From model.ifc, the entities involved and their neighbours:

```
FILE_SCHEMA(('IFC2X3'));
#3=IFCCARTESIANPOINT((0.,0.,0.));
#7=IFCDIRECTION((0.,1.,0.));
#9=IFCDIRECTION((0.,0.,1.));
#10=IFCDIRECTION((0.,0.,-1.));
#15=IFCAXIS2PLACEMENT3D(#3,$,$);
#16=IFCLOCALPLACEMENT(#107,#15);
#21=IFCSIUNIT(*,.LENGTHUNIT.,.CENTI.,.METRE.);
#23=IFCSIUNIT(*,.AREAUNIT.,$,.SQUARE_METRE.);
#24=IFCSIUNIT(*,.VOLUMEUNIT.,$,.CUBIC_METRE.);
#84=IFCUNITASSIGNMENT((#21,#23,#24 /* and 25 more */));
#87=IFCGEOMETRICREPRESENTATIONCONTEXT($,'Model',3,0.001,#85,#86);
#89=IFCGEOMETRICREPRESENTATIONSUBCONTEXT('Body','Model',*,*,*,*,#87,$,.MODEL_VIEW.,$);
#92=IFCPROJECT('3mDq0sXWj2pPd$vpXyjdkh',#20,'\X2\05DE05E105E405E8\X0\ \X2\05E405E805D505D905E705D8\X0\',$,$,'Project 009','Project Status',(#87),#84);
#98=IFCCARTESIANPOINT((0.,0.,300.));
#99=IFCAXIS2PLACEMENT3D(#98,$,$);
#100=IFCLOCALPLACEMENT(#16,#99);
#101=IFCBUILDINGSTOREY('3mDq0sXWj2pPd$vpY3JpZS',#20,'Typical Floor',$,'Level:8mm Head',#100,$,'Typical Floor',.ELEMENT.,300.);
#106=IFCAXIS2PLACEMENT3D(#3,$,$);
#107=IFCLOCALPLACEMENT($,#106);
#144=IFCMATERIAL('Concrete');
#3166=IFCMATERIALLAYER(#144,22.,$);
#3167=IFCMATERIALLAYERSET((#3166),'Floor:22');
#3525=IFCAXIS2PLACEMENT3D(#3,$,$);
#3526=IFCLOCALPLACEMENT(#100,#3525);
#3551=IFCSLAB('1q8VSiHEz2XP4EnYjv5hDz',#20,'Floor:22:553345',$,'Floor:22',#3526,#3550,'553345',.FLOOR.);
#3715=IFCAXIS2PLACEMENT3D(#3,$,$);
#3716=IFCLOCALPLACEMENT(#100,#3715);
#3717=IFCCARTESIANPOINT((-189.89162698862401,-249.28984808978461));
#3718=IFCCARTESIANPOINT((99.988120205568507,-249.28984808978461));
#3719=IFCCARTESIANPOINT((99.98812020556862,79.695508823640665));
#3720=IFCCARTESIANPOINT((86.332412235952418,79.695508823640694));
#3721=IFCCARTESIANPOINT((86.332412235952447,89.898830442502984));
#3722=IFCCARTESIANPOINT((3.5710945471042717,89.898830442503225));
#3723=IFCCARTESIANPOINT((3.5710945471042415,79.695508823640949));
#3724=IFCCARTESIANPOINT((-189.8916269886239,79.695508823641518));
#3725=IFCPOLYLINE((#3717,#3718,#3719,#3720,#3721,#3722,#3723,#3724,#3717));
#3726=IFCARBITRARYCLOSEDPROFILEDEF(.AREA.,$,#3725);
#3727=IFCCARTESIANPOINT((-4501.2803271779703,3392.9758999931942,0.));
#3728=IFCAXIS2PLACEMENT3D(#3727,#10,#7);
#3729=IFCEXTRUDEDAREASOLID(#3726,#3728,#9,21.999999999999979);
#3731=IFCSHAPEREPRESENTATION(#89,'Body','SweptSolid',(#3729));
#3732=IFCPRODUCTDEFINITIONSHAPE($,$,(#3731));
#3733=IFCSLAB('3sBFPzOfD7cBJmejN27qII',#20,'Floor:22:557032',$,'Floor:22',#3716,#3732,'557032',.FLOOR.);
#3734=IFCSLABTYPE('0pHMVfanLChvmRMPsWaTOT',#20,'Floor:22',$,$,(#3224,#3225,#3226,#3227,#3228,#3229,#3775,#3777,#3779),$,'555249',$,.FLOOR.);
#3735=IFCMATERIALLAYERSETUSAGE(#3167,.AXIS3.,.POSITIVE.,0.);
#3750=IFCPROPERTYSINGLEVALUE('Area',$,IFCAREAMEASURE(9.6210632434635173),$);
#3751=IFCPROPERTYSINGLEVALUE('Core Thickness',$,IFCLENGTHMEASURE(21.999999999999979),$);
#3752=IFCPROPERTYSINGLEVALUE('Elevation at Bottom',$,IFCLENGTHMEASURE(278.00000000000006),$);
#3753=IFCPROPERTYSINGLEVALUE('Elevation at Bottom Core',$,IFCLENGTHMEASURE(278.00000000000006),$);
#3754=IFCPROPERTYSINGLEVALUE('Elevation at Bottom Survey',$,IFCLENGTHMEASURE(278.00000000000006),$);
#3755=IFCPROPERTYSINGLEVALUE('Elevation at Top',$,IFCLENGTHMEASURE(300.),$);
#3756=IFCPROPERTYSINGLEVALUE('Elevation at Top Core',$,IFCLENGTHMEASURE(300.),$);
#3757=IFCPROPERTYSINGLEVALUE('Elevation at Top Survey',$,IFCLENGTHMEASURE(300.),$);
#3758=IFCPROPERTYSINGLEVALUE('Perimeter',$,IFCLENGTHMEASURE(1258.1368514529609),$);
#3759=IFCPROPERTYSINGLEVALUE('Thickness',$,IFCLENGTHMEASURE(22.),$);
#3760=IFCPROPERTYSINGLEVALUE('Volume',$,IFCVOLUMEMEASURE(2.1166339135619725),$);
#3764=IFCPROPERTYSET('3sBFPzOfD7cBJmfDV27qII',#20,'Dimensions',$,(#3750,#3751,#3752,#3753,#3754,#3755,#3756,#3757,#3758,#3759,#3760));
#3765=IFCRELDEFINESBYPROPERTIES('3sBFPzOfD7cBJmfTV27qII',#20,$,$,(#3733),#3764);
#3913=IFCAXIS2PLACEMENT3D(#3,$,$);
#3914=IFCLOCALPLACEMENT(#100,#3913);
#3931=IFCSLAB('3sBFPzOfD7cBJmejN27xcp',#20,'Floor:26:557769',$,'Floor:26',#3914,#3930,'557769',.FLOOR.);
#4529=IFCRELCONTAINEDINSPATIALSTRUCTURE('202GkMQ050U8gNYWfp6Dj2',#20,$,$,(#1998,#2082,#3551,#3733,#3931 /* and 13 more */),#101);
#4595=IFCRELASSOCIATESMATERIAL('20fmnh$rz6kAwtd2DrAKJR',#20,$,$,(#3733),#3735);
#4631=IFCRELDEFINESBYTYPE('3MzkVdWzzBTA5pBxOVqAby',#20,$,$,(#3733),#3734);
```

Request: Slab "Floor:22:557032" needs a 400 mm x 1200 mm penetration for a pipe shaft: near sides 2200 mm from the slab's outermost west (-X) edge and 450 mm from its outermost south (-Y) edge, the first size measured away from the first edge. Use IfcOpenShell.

```python
import numpy as np
import ifcopenshell
import ifcopenshell.api.feature
import ifcopenshell.api.geometry
import ifcopenshell.api.pset
import ifcopenshell.api.root
import ifcopenshell.geom
import ifcopenshell.util.element
import ifcopenshell.util.placement
import ifcopenshell.util.representation
import ifcopenshell.util.shape
import ifcopenshell.util.unit

model = ifcopenshell.open("model.ifc")
unit_scale = ifcopenshell.util.unit.calculate_unit_scale(model)
area_scale = ifcopenshell.util.unit.calculate_unit_scale(model, "AREAUNIT")
volume_scale = ifcopenshell.util.unit.calculate_unit_scale(model, "VOLUMEUNIT")
settings = ifcopenshell.geom.settings()


def volume(element):
    """Net volume in cubic metres, openings subtracted."""
    shape = ifcopenshell.geom.create_shape(settings, element)
    return ifcopenshell.util.shape.get_volume(shape.geometry)


slab = model.by_id(3733)
before = volume(slab)

# Extent in the slab's own axes, in metres. The edges named are its -X and -Y sides.
slab_shape = ifcopenshell.geom.create_shape(settings, slab)
vertices = ifcopenshell.util.shape.get_vertices(slab_shape.geometry)
x_min, y_min, bottom = vertices.min(axis=0)
top = vertices[:, 2].max()

opening = ifcopenshell.api.root.create_entity(model, ifc_class="IfcOpeningElement", name="Pipe shaft opening")
context = ifcopenshell.util.representation.get_context(model, "Model", "Body", "MODEL_VIEW")
width, depth = 0.4, 1.2
outline = [(0.0, 0.0), (width, 0.0), (width, depth), (0.0, depth), (0.0, 0.0)]
# Overshoot both faces by 50 mm so the cut is clean.
shape = ifcopenshell.api.geometry.add_slab_representation(
    model, context=context, depth=top - bottom + 0.1, polyline=outline
)
ifcopenshell.api.geometry.assign_representation(model, product=opening, representation=shape)

matrix = ifcopenshell.util.placement.get_local_placement(slab.ObjectPlacement)
matrix[:, 3] = matrix @ np.append(np.array([x_min + 2.2, y_min + 0.45, bottom - 0.05]) / unit_scale, 1.0)
ifcopenshell.api.geometry.edit_object_placement(model, product=opening, matrix=matrix, is_si=False)
ifcopenshell.api.feature.add_feature(model, feature=opening, element=slab)

after = volume(slab)

# Update the slab's stored quantities.
pset = model.by_id(ifcopenshell.util.element.get_pset(slab, "Dimensions", should_inherit=False)["id"])
ifcopenshell.api.pset.edit_pset(model, pset=pset, properties={
    "Area": model.create_entity("IfcAreaMeasure", after / (top - bottom) / area_scale),
    "Volume": model.create_entity("IfcVolumeMeasure", after / volume_scale),
})

print(f"slab volume {before:.3f} -> {after:.3f} m3")

model.write("model_edited.ifc")
```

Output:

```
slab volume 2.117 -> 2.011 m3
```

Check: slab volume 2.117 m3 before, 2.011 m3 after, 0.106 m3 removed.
